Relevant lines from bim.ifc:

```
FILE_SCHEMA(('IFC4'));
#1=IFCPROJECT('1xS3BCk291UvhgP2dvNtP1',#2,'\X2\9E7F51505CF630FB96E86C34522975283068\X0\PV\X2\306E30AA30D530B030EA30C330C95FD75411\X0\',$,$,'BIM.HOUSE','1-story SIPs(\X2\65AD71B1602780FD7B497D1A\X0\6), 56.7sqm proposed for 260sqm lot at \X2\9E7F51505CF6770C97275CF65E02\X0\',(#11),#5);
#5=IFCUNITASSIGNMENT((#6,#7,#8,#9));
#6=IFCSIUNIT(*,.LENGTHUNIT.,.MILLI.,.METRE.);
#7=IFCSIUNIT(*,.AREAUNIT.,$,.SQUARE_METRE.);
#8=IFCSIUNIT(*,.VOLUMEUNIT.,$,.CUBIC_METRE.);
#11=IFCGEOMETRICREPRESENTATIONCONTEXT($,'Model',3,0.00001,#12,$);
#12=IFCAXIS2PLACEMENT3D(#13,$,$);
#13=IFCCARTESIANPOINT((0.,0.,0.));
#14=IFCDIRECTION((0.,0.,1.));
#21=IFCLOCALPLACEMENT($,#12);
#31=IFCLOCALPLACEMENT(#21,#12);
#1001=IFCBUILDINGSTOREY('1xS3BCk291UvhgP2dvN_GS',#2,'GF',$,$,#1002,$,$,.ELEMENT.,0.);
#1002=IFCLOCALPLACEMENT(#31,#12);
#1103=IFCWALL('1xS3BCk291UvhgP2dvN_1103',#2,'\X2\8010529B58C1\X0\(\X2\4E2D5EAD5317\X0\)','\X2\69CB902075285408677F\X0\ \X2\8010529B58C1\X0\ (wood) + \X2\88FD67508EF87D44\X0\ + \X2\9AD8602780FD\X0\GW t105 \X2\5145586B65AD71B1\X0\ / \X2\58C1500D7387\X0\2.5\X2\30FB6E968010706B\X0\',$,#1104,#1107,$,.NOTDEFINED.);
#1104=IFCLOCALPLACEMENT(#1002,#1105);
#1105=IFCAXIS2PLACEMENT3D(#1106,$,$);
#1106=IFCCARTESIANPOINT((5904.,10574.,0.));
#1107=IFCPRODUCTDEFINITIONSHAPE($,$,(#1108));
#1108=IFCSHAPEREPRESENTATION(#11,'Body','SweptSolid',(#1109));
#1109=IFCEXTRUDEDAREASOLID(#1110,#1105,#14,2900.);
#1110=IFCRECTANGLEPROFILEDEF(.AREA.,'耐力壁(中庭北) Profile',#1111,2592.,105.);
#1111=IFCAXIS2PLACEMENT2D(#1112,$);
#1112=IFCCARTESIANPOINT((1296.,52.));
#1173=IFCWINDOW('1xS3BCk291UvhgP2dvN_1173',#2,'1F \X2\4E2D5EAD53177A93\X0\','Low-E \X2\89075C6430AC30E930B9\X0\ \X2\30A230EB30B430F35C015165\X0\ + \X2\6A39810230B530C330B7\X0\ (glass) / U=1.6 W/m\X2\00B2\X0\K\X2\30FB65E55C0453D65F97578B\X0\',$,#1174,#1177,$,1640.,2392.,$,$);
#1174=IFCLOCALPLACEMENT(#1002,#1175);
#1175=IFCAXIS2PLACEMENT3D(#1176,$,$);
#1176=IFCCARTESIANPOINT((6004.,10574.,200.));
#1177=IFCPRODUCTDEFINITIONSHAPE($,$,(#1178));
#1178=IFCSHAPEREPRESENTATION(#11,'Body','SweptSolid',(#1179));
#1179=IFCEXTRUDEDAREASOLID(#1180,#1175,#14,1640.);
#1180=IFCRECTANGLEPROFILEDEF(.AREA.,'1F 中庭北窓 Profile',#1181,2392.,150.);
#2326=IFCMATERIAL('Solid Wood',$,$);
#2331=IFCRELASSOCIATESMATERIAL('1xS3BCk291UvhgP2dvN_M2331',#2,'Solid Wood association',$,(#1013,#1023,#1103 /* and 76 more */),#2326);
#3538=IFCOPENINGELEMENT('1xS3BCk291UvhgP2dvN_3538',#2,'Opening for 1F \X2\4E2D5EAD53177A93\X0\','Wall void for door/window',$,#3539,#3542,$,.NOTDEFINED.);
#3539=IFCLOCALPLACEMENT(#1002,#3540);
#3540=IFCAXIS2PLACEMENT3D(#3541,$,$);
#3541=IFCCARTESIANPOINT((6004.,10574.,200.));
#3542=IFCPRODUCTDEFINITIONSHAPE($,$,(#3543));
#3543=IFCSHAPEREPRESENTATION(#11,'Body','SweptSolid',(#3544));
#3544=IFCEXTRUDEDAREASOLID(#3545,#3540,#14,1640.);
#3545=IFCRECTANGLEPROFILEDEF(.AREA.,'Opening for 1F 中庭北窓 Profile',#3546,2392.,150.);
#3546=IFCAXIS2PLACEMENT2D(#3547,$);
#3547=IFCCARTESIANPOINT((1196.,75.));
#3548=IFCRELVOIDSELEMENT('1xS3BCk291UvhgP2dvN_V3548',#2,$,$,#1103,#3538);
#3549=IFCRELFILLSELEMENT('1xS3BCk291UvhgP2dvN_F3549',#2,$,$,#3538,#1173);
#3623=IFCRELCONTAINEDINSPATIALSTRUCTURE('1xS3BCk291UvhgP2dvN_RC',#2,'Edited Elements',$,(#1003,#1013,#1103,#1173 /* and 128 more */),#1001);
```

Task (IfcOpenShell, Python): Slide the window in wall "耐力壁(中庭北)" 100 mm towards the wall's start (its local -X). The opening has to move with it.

```python
import ifcopenshell
import ifcopenshell.api.geometry
import ifcopenshell.util.placement

model = ifcopenshell.open("bim.ifc")

window = model.by_id(1173)
opening = window.FillsVoids[0].RelatingOpeningElement
wall = opening.VoidsElements[0].RelatingBuildingElement

wall_matrix = ifcopenshell.util.placement.get_local_placement(wall.ObjectPlacement)
shift = wall_matrix[:3, 0] * -100.0
before = ifcopenshell.util.placement.get_local_placement(window.ObjectPlacement)[:3, 3].copy()

# The window is not placed relative to its opening, so move both.
for product in (opening, window):
    matrix = ifcopenshell.util.placement.get_local_placement(product.ObjectPlacement)
    matrix[:3, 3] += shift
    ifcopenshell.api.geometry.edit_object_placement(model, product=product, matrix=matrix, is_si=False)

after = ifcopenshell.util.placement.get_local_placement(window.ObjectPlacement)[:3, 3]
print("window moved by", (after - before).round(3) + 0.0)

model.write("bim_edited.ifc")
```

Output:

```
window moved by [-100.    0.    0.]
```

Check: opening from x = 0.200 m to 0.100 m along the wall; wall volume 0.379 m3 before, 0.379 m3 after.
